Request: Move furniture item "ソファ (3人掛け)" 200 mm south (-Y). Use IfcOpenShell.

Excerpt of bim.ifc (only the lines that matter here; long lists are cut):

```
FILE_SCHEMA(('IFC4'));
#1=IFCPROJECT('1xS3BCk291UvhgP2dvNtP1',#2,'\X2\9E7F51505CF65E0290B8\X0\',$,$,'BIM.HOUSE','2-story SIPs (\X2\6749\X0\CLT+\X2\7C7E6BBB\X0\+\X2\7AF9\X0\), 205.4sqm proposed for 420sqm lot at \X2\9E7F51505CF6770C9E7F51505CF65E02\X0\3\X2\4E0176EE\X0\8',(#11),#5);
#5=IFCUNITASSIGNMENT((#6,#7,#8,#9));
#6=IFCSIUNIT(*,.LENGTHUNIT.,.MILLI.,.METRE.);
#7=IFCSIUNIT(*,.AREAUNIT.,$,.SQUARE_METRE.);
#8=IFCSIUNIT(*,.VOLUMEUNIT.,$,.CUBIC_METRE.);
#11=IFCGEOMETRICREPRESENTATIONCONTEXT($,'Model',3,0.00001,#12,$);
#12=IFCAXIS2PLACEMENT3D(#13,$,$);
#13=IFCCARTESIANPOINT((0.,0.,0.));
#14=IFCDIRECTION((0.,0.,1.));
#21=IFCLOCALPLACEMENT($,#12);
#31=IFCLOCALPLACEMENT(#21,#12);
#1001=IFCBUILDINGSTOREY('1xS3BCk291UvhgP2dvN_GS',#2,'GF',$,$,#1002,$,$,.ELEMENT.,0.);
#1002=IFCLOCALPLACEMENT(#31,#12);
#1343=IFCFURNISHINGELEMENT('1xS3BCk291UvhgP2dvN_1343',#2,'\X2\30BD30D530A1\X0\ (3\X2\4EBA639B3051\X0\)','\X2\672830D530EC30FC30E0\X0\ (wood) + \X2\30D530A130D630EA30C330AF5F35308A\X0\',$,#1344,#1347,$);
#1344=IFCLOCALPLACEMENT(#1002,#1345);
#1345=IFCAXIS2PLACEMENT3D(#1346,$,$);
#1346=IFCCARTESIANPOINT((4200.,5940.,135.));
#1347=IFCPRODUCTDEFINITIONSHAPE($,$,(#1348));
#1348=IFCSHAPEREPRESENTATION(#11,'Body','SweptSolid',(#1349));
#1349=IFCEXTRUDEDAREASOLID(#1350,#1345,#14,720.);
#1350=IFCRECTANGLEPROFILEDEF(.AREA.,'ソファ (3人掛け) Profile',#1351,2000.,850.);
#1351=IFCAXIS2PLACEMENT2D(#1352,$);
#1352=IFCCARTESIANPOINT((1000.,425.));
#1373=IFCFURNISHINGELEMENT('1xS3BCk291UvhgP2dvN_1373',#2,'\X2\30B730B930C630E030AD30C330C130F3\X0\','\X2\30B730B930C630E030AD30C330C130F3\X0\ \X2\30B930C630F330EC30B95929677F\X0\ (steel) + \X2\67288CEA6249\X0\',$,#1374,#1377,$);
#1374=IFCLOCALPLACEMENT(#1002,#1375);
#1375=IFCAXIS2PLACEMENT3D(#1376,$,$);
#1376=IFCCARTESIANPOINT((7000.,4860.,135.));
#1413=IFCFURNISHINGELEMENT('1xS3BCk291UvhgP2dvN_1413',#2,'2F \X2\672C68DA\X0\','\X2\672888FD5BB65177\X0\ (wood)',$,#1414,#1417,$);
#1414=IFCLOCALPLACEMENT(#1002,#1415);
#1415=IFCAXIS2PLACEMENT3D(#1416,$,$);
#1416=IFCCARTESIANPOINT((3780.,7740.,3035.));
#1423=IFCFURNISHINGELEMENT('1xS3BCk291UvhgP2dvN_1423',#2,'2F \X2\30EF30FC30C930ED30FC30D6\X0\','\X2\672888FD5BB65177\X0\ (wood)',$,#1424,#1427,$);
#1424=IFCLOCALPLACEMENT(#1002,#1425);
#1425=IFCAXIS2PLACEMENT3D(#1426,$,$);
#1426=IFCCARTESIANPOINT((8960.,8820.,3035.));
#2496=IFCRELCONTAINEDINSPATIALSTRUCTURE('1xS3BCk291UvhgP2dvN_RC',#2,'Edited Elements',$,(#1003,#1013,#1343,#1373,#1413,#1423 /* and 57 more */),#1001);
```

```python
import ifcopenshell
import ifcopenshell.api.geometry
import ifcopenshell.util.placement

model = ifcopenshell.open("bim.ifc")

item = model.by_id(1343)
matrix = ifcopenshell.util.placement.get_local_placement(item.ObjectPlacement)
matrix[1, 3] -= 200.0
ifcopenshell.api.geometry.edit_object_placement(model, product=item, matrix=matrix, is_si=False)

print(ifcopenshell.util.placement.get_local_placement(item.ObjectPlacement).round(3) + 0.0)

model.write("bim_rev.ifc")
```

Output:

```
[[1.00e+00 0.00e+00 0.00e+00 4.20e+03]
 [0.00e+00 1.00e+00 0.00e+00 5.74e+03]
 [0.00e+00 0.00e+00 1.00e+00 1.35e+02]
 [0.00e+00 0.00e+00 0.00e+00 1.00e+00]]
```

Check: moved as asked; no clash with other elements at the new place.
